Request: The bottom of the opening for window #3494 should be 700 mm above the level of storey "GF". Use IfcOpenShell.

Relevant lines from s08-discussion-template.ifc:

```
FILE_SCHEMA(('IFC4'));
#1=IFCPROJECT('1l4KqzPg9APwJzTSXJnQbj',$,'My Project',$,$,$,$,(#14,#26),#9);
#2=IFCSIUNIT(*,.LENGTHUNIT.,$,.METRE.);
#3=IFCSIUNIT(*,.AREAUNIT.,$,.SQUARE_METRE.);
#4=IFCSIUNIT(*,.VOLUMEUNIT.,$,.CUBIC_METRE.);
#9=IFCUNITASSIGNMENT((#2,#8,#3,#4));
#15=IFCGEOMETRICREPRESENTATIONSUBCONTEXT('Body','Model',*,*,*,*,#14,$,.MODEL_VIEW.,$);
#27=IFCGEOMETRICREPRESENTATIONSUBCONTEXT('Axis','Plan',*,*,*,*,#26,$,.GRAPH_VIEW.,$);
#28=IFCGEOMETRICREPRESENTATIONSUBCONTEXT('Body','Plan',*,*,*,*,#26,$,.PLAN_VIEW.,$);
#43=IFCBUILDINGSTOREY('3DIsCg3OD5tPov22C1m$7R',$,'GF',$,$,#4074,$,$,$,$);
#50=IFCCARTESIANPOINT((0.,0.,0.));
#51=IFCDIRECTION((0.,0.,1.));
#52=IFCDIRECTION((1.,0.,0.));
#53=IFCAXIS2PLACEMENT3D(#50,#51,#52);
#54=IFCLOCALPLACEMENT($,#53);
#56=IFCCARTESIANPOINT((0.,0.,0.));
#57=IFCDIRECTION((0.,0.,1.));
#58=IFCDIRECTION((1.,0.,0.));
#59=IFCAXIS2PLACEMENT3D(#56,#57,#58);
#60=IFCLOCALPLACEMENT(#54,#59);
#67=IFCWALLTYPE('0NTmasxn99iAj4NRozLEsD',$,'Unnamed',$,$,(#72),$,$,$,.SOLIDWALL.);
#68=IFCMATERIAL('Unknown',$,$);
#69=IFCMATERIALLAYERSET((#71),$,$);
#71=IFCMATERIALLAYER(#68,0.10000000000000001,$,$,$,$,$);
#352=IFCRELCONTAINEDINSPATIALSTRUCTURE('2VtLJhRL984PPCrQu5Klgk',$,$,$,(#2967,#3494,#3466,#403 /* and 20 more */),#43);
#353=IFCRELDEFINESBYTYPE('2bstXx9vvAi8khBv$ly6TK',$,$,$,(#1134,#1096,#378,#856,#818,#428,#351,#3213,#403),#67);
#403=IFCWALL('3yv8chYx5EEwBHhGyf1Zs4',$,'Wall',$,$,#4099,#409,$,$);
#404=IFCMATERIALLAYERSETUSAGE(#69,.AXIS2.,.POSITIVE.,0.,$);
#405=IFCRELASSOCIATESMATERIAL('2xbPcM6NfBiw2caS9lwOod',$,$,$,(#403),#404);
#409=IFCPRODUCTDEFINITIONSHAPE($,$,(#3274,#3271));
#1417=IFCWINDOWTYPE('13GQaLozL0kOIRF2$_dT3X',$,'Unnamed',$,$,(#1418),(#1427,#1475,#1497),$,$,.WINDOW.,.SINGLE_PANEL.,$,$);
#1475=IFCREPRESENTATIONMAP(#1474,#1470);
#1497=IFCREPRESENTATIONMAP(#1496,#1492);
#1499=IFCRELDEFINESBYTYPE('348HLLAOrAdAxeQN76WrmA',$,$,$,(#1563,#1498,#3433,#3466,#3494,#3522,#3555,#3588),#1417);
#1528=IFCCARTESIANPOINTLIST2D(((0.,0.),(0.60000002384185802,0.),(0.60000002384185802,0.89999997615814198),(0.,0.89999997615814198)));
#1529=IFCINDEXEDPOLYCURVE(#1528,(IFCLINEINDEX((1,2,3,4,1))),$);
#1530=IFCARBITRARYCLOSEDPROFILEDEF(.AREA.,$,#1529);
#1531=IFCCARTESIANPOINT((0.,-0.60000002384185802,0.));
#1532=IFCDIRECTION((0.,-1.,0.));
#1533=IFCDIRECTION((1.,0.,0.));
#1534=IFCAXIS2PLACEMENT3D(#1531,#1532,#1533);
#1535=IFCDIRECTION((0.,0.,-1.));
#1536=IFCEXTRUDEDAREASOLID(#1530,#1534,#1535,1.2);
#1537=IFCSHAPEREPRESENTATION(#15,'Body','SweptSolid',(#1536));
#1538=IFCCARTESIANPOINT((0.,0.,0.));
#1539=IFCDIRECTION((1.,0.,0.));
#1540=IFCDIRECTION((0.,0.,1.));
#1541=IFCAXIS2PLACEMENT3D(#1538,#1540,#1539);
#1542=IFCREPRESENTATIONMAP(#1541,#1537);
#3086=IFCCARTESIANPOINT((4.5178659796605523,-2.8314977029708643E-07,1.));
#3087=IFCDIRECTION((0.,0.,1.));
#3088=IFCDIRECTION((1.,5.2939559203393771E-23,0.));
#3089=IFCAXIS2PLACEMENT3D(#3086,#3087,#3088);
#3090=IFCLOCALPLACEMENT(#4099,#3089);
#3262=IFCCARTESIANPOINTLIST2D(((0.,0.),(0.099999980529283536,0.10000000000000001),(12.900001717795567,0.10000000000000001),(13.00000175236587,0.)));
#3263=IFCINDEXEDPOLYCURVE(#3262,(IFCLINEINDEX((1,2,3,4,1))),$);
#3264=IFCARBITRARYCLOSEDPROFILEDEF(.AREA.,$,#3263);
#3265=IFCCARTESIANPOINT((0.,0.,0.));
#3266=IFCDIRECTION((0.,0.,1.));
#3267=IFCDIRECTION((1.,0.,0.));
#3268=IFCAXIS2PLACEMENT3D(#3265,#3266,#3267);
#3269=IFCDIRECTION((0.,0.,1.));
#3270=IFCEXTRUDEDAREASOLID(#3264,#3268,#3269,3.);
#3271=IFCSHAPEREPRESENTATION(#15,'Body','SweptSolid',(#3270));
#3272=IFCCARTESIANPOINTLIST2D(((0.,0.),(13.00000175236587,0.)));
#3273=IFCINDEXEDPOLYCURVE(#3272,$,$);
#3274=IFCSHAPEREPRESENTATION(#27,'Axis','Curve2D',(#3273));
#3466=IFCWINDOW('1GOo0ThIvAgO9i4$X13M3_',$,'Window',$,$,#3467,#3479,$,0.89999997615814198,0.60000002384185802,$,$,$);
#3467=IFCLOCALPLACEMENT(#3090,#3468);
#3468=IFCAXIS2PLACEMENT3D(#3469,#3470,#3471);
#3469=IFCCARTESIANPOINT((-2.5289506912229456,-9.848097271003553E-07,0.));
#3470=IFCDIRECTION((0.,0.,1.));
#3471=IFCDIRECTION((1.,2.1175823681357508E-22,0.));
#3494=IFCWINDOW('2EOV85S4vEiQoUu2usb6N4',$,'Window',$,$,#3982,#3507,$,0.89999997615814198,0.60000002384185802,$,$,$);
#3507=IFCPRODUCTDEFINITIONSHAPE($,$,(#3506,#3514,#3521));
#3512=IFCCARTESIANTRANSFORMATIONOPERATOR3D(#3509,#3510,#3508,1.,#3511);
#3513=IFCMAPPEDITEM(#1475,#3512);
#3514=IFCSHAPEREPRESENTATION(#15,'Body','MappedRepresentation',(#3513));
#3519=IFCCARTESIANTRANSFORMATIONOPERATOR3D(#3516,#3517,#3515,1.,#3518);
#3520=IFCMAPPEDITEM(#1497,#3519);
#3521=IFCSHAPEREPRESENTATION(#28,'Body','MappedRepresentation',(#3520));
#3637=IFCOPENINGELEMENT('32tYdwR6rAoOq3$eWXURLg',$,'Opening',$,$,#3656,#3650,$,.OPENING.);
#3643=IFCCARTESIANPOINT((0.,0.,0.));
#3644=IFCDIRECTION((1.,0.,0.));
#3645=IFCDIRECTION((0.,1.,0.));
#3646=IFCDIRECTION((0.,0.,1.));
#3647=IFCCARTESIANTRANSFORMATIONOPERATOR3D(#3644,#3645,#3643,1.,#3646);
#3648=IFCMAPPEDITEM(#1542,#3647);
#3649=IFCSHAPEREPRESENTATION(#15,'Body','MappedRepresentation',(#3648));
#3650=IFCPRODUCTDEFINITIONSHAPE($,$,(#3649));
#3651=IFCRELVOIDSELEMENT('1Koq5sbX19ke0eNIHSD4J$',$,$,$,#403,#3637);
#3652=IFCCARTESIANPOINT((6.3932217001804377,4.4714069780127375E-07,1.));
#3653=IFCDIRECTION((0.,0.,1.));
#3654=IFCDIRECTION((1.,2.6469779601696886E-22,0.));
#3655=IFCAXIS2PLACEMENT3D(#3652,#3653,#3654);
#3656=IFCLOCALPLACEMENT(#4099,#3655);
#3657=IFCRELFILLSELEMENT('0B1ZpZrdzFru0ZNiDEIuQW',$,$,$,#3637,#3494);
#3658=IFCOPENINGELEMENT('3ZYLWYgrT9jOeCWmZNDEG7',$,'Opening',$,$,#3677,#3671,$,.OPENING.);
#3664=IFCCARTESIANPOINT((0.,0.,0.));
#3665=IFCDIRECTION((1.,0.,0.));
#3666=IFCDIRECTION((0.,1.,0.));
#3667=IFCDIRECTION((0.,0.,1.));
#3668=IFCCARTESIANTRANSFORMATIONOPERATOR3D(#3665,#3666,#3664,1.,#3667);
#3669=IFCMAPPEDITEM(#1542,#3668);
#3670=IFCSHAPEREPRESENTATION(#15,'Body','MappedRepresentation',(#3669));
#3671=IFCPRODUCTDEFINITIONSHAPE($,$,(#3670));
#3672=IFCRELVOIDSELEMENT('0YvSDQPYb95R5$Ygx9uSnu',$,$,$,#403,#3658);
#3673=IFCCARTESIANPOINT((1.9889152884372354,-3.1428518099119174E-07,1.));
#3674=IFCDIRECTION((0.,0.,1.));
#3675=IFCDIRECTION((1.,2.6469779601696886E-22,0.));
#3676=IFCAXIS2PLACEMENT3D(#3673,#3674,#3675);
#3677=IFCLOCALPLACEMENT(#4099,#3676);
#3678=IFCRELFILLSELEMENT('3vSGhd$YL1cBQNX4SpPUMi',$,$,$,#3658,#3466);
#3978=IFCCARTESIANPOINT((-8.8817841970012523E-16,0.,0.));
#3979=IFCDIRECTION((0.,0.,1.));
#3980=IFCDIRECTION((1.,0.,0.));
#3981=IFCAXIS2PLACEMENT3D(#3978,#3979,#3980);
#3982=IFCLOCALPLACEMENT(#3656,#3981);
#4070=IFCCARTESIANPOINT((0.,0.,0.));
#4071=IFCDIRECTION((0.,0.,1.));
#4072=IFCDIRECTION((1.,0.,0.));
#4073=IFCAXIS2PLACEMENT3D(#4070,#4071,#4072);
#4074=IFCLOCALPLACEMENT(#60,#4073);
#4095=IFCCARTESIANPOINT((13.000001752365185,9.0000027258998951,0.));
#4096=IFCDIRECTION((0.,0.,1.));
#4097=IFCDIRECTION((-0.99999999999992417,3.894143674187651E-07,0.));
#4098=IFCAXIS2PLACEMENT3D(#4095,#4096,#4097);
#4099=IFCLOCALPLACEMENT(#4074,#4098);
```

```python
import numpy as np
import ifcopenshell
import ifcopenshell.api.geometry
import ifcopenshell.geom
import ifcopenshell.util.element
import ifcopenshell.util.placement
import ifcopenshell.util.shape
import ifcopenshell.util.unit

model = ifcopenshell.open("s08-discussion-template.ifc")
unit_scale = ifcopenshell.util.unit.calculate_unit_scale(model)

window = model.by_guid("2EOV85S4vEiQoUu2usb6N4")
opening = window.FillsVoids[0].RelatingOpeningElement
storey = ifcopenshell.util.element.get_container(window, ifc_class="IfcBuildingStorey")
level = ifcopenshell.util.placement.get_local_placement(storey.ObjectPlacement)[2, 3]

# The opening's origin need not be at the sill, so measure its lowest point.
shape = ifcopenshell.geom.create_shape(ifcopenshell.geom.settings(), opening)
bottom = ifcopenshell.util.shape.get_shape_bottom_elevation(shape, shape.geometry) / unit_scale
dz = level + 0.7 - bottom

shift = np.array([0.0, 0.0, dz])
# The window is placed relative to its opening, so it follows when the opening moves.
matrix = ifcopenshell.util.placement.get_local_placement(opening.ObjectPlacement)
matrix[:3, 3] += shift
ifcopenshell.api.geometry.edit_object_placement(
    model, product=opening, matrix=matrix, is_si=False, should_transform_children=True
)

print(f"moved by {dz * unit_scale:+.3f} m")

model.write("s08-discussion-template_updated.ifc")
```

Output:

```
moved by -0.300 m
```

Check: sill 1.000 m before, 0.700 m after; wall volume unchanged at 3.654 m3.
